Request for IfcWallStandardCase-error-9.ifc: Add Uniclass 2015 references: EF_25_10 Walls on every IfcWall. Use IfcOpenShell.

First a look at what the model holds.

```python
import ifcopenshell

model = ifcopenshell.open("IfcWallStandardCase-error-9.ifc")
print(model.schema)
print("classifications:", [c.Name for c in model.by_type("IfcClassification")])
for ifc_class in ("IfcDoor", "IfcRoof", "IfcStair", "IfcWall", "IfcWindow"):
    print(ifc_class, len(model.by_type(ifc_class)))
```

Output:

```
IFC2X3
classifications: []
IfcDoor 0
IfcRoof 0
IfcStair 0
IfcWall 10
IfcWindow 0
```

```python
import ifcopenshell
import ifcopenshell.api.classification

model = ifcopenshell.open("IfcWallStandardCase-error-9.ifc")

# IFC2X3 requires Source and Edition and has no link from the project to the system.
system = model.create_entity("IfcClassification", Source="NBS", Edition="2015", Name="Uniclass 2015")

codes = {
    "IfcWall": ("EF_25_10", "Walls"),
}
for ifc_class, (code, name) in codes.items():
    products = model.by_type(ifc_class)
    ifcopenshell.api.classification.add_reference(
        model, products=products, classification=system, identification=code, name=name
    )
    print(code, len(products))

model.write("IfcWallStandardCase-error-9_edited.ifc")
```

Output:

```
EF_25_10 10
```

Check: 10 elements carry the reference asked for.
